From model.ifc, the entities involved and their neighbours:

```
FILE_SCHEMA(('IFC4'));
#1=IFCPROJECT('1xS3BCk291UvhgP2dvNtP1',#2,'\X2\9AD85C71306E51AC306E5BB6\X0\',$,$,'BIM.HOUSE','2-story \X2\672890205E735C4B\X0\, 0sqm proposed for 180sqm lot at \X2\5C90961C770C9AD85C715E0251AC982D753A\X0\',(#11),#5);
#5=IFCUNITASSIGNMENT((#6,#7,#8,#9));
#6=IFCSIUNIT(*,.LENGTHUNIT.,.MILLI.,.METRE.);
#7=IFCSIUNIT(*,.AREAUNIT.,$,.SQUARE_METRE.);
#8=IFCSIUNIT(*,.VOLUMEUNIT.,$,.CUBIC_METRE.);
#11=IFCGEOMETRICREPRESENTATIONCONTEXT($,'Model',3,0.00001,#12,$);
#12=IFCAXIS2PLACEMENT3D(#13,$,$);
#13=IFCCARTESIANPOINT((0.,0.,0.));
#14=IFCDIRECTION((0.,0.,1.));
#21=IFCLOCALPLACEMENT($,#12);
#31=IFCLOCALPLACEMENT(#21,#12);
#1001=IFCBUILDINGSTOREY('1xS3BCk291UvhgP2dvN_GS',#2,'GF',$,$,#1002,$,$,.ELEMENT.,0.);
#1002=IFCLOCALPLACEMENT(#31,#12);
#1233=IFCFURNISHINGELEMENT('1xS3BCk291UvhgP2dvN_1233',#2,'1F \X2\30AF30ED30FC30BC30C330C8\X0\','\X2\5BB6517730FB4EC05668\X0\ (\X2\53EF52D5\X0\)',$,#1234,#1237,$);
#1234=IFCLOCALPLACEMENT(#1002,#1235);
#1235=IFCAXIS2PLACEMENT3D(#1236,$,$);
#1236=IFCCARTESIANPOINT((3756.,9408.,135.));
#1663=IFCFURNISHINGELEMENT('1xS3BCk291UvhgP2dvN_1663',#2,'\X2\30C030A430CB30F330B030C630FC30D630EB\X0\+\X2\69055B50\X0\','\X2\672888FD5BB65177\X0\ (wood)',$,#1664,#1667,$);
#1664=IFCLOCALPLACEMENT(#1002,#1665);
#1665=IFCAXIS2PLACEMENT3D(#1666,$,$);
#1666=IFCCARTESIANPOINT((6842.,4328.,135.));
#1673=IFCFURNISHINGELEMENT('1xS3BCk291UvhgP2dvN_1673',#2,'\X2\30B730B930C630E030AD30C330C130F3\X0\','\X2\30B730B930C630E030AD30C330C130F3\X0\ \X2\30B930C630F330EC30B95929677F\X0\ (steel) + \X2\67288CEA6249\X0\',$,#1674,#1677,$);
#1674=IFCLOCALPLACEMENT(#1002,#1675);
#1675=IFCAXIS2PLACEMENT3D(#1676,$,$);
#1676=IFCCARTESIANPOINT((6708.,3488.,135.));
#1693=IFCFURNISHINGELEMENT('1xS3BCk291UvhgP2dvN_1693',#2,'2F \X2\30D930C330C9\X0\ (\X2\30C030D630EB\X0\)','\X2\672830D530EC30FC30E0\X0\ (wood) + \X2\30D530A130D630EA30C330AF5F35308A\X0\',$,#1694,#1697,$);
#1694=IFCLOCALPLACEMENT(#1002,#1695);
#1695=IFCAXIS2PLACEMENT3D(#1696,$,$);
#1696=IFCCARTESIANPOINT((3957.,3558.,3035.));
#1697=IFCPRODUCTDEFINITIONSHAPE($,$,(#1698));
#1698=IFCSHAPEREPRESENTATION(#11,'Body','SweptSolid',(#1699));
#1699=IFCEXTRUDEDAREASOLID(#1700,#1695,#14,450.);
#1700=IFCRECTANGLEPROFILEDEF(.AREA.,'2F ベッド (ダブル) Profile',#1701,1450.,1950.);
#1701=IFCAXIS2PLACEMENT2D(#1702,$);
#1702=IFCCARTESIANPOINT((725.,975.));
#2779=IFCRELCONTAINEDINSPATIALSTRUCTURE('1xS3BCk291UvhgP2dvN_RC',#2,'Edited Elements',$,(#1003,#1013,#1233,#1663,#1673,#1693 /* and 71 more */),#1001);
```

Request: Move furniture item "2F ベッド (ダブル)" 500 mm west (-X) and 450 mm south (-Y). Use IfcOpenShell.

```python
import ifcopenshell
import ifcopenshell.api.geometry
import ifcopenshell.util.placement
import ifcopenshell.util.unit

model = ifcopenshell.open("model.ifc")
unit_scale = ifcopenshell.util.unit.calculate_unit_scale(model)

item = model.by_guid("1xS3BCk291UvhgP2dvN_1693")
matrix = ifcopenshell.util.placement.get_local_placement(item.ObjectPlacement)
matrix[0, 3] -= 0.5 / unit_scale
matrix[1, 3] -= 0.45 / unit_scale
ifcopenshell.api.geometry.edit_object_placement(model, product=item, matrix=matrix, is_si=False)

print(ifcopenshell.util.placement.get_local_placement(item.ObjectPlacement).round(3) + 0.0)

model.write("model_updated.ifc")
```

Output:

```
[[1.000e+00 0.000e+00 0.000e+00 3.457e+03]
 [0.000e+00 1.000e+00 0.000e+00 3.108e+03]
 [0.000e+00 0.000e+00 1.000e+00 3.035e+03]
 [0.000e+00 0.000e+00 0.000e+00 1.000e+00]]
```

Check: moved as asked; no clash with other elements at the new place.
